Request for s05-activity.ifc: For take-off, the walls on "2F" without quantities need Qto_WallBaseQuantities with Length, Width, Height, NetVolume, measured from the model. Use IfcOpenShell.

First a look at what the model holds.

```python
import ifcopenshell
import ifcopenshell.util.element
import ifcopenshell.util.unit

model = ifcopenshell.open("s05-activity.ifc")
print(model.schema)
for unit_type in ("LENGTHUNIT", "AREAUNIT", "VOLUMEUNIT"):
    print(unit_type, ifcopenshell.util.unit.calculate_unit_scale(model, unit_type))
storey = next(s for s in model.by_type("IfcBuildingStorey") if s.Name == "2F")
walls = [e for e in ifcopenshell.util.element.get_decomposition(storey) if e.is_a("IfcWall")]
for e in sorted(walls, key=lambda e: e.id()):
    print(e.id(), e.is_a(), e.Name, list(ifcopenshell.util.element.get_psets(e, qtos_only=True)), sep=" | ")
```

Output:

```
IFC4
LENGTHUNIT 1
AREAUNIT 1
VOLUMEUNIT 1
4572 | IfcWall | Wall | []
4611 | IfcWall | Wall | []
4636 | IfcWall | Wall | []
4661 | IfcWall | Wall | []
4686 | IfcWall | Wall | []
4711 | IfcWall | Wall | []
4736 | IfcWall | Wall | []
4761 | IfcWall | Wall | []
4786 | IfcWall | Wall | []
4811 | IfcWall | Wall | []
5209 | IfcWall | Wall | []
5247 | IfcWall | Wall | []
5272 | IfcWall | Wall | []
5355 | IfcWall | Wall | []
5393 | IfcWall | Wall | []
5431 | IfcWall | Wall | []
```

```python
import ifcopenshell
import ifcopenshell.api.pset
import ifcopenshell.geom
import ifcopenshell.util.element
import ifcopenshell.util.shape
import ifcopenshell.util.unit

model = ifcopenshell.open("s05-activity.ifc")
unit_scale = ifcopenshell.util.unit.calculate_unit_scale(model)
volume_scale = ifcopenshell.util.unit.calculate_unit_scale(model, "VOLUMEUNIT")
settings = ifcopenshell.geom.settings()

storey = next(s for s in model.by_type("IfcBuildingStorey") if s.Name == "2F")
walls = [e for e in ifcopenshell.util.element.get_decomposition(storey) if e.is_a("IfcWall")]

for e in sorted(walls, key=lambda e: e.id()):
    if ifcopenshell.util.element.get_psets(e, qtos_only=True, should_inherit=False):
        continue
    # Geometry comes back in metres, in the element's own axes.
    shape = ifcopenshell.geom.create_shape(settings, e)
    values = {
        "Length": ifcopenshell.util.shape.get_x(shape.geometry) / unit_scale,
        "Width": ifcopenshell.util.shape.get_y(shape.geometry) / unit_scale,
        "Height": ifcopenshell.util.shape.get_z(shape.geometry) / unit_scale,
        "NetVolume": ifcopenshell.util.shape.get_volume(shape.geometry) / volume_scale,
    }
    qto = ifcopenshell.api.pset.add_qto(model, product=e, name="Qto_WallBaseQuantities")
    ifcopenshell.api.pset.edit_qto(model, qto=qto, properties=values)
    print(e.id(), {k: round(v, 3) for k, v in values.items()})

model.write("s05-activity_updated.ifc")
```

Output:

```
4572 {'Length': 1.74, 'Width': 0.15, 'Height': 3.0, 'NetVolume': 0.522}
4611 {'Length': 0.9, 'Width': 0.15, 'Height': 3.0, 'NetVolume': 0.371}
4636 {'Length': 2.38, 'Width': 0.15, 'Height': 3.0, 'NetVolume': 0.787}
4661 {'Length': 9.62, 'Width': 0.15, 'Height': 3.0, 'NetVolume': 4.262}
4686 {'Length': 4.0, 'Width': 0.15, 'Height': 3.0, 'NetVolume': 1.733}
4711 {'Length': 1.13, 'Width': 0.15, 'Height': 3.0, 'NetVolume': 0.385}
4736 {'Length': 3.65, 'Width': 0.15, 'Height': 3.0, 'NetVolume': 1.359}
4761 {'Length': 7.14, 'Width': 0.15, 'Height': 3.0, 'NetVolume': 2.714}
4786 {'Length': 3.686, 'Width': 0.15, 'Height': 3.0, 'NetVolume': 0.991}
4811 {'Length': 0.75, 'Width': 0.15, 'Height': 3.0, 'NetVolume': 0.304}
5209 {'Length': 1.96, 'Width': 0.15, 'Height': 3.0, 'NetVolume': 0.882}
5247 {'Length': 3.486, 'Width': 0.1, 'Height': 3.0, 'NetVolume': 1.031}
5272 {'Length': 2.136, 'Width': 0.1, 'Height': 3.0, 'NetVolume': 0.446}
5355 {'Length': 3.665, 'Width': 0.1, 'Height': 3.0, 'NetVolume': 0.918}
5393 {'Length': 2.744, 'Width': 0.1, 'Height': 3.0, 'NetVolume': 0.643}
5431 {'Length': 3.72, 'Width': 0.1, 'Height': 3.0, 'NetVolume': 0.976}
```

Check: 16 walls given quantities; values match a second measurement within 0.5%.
